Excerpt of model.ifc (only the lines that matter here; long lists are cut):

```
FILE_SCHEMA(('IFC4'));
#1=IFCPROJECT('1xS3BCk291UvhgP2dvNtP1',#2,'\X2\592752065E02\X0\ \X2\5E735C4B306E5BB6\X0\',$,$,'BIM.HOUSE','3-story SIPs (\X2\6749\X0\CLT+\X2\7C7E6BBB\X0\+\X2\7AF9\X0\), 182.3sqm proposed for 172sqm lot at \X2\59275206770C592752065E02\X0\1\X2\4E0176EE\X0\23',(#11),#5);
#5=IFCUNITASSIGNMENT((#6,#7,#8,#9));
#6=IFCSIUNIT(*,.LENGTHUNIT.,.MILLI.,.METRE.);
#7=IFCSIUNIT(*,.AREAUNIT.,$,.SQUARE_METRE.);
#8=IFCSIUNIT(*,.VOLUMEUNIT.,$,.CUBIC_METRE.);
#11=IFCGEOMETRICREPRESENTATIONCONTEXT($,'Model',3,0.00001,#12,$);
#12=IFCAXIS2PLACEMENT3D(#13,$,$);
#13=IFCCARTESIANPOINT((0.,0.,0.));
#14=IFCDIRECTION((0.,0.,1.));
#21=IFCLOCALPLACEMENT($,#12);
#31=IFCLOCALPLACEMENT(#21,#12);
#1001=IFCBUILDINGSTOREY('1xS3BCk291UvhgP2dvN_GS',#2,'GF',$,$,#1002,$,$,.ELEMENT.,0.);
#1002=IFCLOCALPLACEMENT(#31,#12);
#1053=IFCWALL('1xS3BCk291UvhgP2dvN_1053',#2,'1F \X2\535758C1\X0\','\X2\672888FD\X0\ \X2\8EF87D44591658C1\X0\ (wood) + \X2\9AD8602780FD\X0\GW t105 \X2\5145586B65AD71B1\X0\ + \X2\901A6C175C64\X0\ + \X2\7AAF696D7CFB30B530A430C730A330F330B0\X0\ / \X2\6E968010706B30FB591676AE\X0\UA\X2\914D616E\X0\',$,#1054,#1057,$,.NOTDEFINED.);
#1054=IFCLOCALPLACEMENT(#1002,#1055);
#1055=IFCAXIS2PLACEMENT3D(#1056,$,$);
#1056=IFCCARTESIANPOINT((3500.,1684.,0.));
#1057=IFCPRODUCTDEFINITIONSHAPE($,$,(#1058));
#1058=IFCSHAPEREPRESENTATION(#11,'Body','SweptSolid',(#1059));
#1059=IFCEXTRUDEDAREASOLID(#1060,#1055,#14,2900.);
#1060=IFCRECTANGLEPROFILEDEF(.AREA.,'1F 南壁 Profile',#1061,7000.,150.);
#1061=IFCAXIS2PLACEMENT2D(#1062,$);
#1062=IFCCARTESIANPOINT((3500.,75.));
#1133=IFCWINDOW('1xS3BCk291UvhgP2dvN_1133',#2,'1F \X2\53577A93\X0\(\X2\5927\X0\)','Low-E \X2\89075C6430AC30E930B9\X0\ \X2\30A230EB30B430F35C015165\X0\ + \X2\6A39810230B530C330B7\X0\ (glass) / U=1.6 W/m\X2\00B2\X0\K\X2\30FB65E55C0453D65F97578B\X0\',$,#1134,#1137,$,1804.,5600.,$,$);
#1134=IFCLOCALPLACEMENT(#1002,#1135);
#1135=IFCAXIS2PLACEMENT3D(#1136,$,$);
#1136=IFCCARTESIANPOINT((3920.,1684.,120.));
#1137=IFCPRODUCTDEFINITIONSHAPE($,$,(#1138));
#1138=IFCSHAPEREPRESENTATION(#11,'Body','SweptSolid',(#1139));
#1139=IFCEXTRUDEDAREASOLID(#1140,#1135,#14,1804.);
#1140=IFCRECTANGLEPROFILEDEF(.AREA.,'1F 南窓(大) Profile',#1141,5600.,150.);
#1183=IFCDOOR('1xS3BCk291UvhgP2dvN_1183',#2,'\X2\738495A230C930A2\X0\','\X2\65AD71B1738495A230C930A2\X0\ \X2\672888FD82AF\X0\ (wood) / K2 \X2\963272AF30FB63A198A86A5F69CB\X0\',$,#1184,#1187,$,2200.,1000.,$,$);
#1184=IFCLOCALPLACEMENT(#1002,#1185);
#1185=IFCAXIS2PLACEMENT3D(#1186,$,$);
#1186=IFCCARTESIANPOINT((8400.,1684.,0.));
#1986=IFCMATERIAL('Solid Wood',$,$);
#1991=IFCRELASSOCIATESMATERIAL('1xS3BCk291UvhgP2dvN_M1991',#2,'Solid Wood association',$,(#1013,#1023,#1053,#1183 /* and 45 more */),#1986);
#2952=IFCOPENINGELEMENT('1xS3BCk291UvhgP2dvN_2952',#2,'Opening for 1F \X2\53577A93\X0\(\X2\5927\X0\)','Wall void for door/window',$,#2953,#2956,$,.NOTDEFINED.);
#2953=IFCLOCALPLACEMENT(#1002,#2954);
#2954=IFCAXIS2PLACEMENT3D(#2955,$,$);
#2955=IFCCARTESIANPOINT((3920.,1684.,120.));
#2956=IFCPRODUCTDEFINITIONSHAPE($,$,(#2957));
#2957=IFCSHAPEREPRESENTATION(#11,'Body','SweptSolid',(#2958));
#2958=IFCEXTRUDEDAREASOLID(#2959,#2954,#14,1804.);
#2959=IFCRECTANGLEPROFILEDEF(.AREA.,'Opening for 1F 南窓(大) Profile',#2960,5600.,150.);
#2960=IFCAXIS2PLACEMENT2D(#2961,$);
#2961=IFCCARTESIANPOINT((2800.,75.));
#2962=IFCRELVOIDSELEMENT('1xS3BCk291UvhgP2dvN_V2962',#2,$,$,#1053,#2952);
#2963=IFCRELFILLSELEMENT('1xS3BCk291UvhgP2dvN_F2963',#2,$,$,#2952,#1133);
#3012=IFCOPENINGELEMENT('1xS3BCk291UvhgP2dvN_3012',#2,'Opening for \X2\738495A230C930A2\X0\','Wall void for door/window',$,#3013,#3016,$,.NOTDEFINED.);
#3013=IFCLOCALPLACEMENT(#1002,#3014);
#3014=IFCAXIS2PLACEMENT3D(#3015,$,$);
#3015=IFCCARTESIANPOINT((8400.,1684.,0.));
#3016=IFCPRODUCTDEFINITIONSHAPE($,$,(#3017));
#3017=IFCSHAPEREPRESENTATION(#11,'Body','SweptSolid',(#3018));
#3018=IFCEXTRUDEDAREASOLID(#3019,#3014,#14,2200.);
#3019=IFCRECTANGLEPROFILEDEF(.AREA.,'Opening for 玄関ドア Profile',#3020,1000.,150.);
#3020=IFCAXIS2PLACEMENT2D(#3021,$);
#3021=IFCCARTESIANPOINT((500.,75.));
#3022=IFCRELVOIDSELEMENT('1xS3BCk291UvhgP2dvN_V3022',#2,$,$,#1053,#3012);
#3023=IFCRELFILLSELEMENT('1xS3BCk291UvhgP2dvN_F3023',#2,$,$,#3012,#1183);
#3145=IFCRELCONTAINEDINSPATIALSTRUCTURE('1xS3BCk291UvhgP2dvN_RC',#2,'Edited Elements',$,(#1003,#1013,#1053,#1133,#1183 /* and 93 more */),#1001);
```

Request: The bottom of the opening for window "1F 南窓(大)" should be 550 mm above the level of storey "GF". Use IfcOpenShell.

```python
import numpy as np
import ifcopenshell
import ifcopenshell.api.geometry
import ifcopenshell.geom
import ifcopenshell.util.element
import ifcopenshell.util.placement
import ifcopenshell.util.shape
import ifcopenshell.util.unit

model = ifcopenshell.open("model.ifc")
unit_scale = ifcopenshell.util.unit.calculate_unit_scale(model)

window = model.by_id(1133)
opening = window.FillsVoids[0].RelatingOpeningElement
storey = ifcopenshell.util.element.get_container(window, ifc_class="IfcBuildingStorey")
level = ifcopenshell.util.placement.get_local_placement(storey.ObjectPlacement)[2, 3]

# The opening's origin need not be at the sill, so measure its lowest point.
shape = ifcopenshell.geom.create_shape(ifcopenshell.geom.settings(), opening)
bottom = ifcopenshell.util.shape.get_shape_bottom_elevation(shape, shape.geometry) / unit_scale
dz = level + 0.55 / unit_scale - bottom

shift = np.array([0.0, 0.0, dz])
# The window is not placed relative to its opening, so move both.
for product in (opening, window):
    matrix = ifcopenshell.util.placement.get_local_placement(product.ObjectPlacement)
    matrix[:3, 3] += shift
    ifcopenshell.api.geometry.edit_object_placement(model, product=product, matrix=matrix, is_si=False)

print(f"moved by {dz * unit_scale:+.3f} m")

model.write("model_edited.ifc")
```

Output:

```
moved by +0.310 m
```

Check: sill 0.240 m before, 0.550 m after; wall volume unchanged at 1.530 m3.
